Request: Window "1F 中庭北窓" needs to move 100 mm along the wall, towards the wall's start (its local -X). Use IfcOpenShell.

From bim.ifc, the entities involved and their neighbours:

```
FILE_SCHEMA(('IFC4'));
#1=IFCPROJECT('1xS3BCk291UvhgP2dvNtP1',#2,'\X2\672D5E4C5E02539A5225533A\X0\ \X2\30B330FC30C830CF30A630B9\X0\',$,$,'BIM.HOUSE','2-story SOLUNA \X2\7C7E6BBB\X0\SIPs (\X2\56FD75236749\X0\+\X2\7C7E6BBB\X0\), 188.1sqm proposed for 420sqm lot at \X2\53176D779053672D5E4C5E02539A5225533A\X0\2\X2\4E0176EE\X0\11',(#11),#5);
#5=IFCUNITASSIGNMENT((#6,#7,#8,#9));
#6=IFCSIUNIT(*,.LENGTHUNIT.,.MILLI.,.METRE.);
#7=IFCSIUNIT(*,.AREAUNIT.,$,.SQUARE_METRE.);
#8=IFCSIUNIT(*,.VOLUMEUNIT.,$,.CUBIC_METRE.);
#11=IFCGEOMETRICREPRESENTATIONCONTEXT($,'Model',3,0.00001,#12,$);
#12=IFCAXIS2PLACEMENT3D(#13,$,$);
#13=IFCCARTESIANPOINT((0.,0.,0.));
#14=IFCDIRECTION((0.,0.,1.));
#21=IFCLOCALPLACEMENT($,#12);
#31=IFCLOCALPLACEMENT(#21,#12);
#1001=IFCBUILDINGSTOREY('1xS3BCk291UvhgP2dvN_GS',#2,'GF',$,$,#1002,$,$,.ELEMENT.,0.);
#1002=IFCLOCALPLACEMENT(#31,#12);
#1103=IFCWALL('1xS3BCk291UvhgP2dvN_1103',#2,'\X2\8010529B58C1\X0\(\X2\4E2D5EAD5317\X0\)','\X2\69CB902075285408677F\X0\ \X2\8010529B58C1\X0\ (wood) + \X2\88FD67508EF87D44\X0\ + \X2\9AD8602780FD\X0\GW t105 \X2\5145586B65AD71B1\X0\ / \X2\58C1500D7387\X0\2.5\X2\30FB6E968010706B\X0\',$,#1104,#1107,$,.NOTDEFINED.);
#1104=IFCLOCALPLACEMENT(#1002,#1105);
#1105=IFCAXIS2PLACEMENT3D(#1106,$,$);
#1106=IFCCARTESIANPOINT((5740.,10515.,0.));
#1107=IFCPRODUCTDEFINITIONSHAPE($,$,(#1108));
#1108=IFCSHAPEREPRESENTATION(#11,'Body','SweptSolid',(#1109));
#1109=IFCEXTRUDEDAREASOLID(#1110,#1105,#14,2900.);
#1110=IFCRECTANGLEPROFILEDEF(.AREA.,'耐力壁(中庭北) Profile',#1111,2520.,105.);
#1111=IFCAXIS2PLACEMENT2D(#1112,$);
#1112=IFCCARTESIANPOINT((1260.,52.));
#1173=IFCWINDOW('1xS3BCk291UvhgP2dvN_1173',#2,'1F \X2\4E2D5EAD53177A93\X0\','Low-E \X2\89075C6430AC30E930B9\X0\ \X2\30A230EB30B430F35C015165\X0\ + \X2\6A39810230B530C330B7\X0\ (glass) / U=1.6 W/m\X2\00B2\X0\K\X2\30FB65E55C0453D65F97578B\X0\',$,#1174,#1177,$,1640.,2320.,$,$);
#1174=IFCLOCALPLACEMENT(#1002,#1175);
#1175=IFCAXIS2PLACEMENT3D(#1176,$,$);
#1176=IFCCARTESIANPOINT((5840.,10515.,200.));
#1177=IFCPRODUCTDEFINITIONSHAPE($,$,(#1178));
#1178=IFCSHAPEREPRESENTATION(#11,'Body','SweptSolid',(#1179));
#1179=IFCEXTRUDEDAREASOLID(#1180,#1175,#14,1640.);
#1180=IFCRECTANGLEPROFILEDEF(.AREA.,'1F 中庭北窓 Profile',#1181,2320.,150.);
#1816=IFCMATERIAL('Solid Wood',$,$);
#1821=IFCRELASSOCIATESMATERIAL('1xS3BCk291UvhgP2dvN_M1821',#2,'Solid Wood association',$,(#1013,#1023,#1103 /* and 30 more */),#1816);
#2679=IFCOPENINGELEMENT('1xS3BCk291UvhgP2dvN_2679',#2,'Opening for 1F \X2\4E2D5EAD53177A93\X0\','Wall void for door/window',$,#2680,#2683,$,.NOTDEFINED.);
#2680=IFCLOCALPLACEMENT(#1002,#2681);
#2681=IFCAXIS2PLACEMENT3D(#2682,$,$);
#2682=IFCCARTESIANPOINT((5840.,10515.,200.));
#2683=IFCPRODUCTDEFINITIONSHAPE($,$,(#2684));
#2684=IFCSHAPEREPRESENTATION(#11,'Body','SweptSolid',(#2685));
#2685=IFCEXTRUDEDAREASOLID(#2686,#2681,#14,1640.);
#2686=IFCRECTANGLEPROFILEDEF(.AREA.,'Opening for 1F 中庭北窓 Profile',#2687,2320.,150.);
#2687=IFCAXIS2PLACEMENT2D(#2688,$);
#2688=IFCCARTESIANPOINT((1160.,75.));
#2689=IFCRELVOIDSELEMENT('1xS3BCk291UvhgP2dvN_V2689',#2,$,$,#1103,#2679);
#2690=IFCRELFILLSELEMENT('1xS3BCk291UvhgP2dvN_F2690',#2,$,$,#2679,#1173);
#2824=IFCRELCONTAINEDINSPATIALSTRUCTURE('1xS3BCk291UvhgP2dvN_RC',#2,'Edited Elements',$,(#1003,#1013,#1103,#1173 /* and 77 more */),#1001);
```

```python
import ifcopenshell
import ifcopenshell.api.geometry
import ifcopenshell.util.placement

model = ifcopenshell.open("bim.ifc")

window = model.by_guid("1xS3BCk291UvhgP2dvN_1173")
opening = window.FillsVoids[0].RelatingOpeningElement
wall = opening.VoidsElements[0].RelatingBuildingElement

wall_matrix = ifcopenshell.util.placement.get_local_placement(wall.ObjectPlacement)
shift = wall_matrix[:3, 0] * -100.0
before = ifcopenshell.util.placement.get_local_placement(window.ObjectPlacement)[:3, 3].copy()

# The window is not placed relative to its opening, so move both.
for product in (opening, window):
    matrix = ifcopenshell.util.placement.get_local_placement(product.ObjectPlacement)
    matrix[:3, 3] += shift
    ifcopenshell.api.geometry.edit_object_placement(model, product=product, matrix=matrix, is_si=False)

after = ifcopenshell.util.placement.get_local_placement(window.ObjectPlacement)[:3, 3]
print("window moved by", (after - before).round(3) + 0.0)

model.write("bim-out.ifc")
```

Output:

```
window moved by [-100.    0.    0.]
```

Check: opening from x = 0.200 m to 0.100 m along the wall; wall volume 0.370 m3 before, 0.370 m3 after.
